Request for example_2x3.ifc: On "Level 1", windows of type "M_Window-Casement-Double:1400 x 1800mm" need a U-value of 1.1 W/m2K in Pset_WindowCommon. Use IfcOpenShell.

First a look at what the model holds.

```python
import ifcopenshell
import ifcopenshell.util.element

model = ifcopenshell.open("example_2x3.ifc")
print(model.schema)
storey = next(s for s in model.by_type("IfcBuildingStorey") if s.Name == "Level 1")
windows = [e for e in ifcopenshell.util.element.get_decomposition(storey) if e.is_a("IfcWindow")]
seen = {}
for e in windows:
    element_type = ifcopenshell.util.element.get_type(e)
    key = (element_type.Name if element_type != e and element_type else None, ifcopenshell.util.element.get_pset(e, "Pset_WindowCommon", "ThermalTransmittance"))
    seen[key] = seen.get(key, 0) + 1
for (name, value), count in sorted(seen.items(), key=str):
    print(count, "x", name, "|", value)
```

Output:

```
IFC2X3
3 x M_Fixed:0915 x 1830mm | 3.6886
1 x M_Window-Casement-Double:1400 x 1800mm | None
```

```python
import ifcopenshell
import ifcopenshell.api.pset
import ifcopenshell.util.element

model = ifcopenshell.open("example_2x3.ifc")

storey = next(s for s in model.by_type("IfcBuildingStorey") if s.Name == "Level 1")
windows = [e for e in ifcopenshell.util.element.get_decomposition(storey) if e.is_a("IfcWindow")]

count = 0
for e in windows:
    element_type = ifcopenshell.util.element.get_type(e)
    if element_type in (None, e) or element_type.Name != "M_Window-Casement-Double:1400 x 1800mm":
        continue
    # add_pset returns the element's existing set when there is one.
    pset = ifcopenshell.api.pset.add_pset(model, product=e, name="Pset_WindowCommon")
    ifcopenshell.api.pset.edit_pset(model, pset=pset, properties={"ThermalTransmittance": 1.1})
    count += 1

print(count, "windows updated")

model.write("example_2x3_edited.ifc")
```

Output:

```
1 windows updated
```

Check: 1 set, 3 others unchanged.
